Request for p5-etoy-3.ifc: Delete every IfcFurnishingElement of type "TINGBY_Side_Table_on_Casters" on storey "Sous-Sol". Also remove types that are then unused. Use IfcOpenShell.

First a look at what the model holds.

```python
import ifcopenshell
import ifcopenshell.util.element

model = ifcopenshell.open("p5-etoy-3.ifc")
print(model.schema)
storey = next(s for s in model.by_type("IfcBuildingStorey") if s.Name == "Sous-Sol")
furniture = [e for e in ifcopenshell.util.element.get_decomposition(storey) if e.is_a("IfcFurnishingElement")]
seen = {}
for e in furniture:
    element_type = ifcopenshell.util.element.get_type(e)
    name = element_type.Name if element_type not in (None, e) else None
    seen[name] = seen.get(name, 0) + 1
for name, count in sorted(seen.items(), key=str):
    print(count, "x", name)
```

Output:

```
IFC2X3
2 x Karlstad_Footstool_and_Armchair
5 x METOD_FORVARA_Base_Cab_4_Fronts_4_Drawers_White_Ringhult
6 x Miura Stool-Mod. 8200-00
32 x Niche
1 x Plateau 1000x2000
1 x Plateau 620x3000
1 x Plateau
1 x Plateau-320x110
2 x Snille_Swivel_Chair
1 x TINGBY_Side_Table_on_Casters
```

```python
import ifcopenshell
import ifcopenshell.api.root
import ifcopenshell.util.element

model = ifcopenshell.open("p5-etoy-3.ifc")

storey = next(s for s in model.by_type("IfcBuildingStorey") if s.Name == "Sous-Sol")
furniture = [e for e in ifcopenshell.util.element.get_decomposition(storey) if e.is_a("IfcFurnishingElement")]
targets = [e for e in furniture if (t := ifcopenshell.util.element.get_type(e)) not in (None, e) and t.Name == "TINGBY_Side_Table_on_Casters"]
types = {ifcopenshell.util.element.get_type(e) for e in targets} - {None, *targets}

for e in targets:
    ifcopenshell.api.root.remove_product(model, product=e)
print(len(targets), "removed")

unused = [t for t in types if not ifcopenshell.util.element.get_types(t)]
for t in unused:
    ifcopenshell.api.root.remove_product(model, product=t)
print(len(unused), "unused types removed")

model.write("p5-etoy-3_edited.ifc")
```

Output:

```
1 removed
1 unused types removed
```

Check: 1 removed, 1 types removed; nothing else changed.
